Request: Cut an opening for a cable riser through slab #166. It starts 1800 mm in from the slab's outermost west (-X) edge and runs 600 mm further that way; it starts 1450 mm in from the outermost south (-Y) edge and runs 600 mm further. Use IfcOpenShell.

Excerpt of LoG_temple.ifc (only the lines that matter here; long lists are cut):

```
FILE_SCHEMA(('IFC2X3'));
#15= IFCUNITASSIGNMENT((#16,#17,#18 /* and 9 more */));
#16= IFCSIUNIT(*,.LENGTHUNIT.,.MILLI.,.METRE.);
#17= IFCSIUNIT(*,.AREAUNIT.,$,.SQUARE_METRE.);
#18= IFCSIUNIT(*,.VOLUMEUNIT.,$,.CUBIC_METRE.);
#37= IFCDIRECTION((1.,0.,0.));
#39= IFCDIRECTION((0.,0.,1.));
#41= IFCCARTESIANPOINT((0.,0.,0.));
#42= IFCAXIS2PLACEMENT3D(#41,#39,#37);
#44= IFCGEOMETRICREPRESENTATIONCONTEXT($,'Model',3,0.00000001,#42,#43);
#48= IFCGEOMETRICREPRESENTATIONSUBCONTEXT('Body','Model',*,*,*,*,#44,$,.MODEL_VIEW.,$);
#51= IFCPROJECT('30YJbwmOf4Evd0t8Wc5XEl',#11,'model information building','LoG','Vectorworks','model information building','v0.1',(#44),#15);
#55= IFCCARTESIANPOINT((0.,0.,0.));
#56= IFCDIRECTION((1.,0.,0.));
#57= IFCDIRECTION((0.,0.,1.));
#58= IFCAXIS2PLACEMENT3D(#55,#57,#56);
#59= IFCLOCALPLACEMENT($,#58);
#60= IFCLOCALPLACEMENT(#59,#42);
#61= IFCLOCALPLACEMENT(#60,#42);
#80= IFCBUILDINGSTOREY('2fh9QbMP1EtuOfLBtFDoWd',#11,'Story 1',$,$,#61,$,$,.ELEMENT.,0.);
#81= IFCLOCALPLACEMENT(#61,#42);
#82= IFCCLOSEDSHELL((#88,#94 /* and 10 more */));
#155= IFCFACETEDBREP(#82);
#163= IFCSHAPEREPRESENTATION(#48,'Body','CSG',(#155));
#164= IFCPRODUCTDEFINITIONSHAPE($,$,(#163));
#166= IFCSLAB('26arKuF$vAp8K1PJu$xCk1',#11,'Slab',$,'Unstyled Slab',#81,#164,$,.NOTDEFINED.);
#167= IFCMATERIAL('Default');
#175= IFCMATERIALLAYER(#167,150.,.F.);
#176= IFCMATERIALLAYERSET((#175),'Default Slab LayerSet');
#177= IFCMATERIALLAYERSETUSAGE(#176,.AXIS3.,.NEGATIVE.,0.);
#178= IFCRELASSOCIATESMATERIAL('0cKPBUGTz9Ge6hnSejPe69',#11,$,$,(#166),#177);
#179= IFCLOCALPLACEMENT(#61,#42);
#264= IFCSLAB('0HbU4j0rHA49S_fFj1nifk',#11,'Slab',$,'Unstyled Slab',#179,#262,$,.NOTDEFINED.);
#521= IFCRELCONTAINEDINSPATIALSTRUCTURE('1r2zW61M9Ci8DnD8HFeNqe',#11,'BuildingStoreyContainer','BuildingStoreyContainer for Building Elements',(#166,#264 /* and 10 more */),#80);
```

```python
import numpy as np
import ifcopenshell
import ifcopenshell.api.feature
import ifcopenshell.api.geometry
import ifcopenshell.api.root
import ifcopenshell.geom
import ifcopenshell.util.placement
import ifcopenshell.util.representation
import ifcopenshell.util.shape
import ifcopenshell.util.unit

model = ifcopenshell.open("LoG_temple.ifc")
unit_scale = ifcopenshell.util.unit.calculate_unit_scale(model)
settings = ifcopenshell.geom.settings()


def volume(element):
    """Net volume in cubic metres, openings subtracted."""
    shape = ifcopenshell.geom.create_shape(settings, element)
    return ifcopenshell.util.shape.get_volume(shape.geometry)


slab = model.by_id(166)
before = volume(slab)

# Extent in the slab's own axes, in metres. The edges named are its -X and -Y sides.
slab_shape = ifcopenshell.geom.create_shape(settings, slab)
vertices = ifcopenshell.util.shape.get_vertices(slab_shape.geometry)
x_min, y_min, bottom = vertices.min(axis=0)
top = vertices[:, 2].max()

opening = ifcopenshell.api.root.create_entity(model, ifc_class="IfcOpeningElement", name="Cable riser opening")
context = ifcopenshell.util.representation.get_context(model, "Model", "Body", "MODEL_VIEW")
width, depth = 0.6, 0.6
outline = [(0.0, 0.0), (width, 0.0), (width, depth), (0.0, depth), (0.0, 0.0)]
# Overshoot both faces by 50 mm so the cut is clean.
shape = ifcopenshell.api.geometry.add_slab_representation(
    model, context=context, depth=top - bottom + 0.1, polyline=outline
)
ifcopenshell.api.geometry.assign_representation(model, product=opening, representation=shape)

matrix = ifcopenshell.util.placement.get_local_placement(slab.ObjectPlacement)
matrix[:, 3] = matrix @ np.append(np.array([x_min + 1.8, y_min + 1.45, bottom - 0.05]) / unit_scale, 1.0)
ifcopenshell.api.geometry.edit_object_placement(model, product=opening, matrix=matrix, is_si=False)
ifcopenshell.api.feature.add_feature(model, feature=opening, element=slab)

after = volume(slab)

print(f"slab volume {before:.3f} -> {after:.3f} m3")

model.write("LoG_temple_edited.ifc")
```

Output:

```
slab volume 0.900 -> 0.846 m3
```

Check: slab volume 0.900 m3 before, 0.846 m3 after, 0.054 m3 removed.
